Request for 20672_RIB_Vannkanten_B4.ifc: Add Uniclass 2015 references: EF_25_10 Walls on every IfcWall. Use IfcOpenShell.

First a look at what the model holds.

```python
import ifcopenshell

model = ifcopenshell.open("20672_RIB_Vannkanten_B4.ifc")
print(model.schema)
print("classifications:", [c.Name for c in model.by_type("IfcClassification")])
for ifc_class in ("IfcDoor", "IfcRoof", "IfcStair", "IfcWall", "IfcWindow"):
    print(ifc_class, len(model.by_type(ifc_class)))
```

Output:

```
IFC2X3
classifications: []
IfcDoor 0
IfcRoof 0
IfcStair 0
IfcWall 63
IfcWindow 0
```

```python
import ifcopenshell
import ifcopenshell.api.classification

model = ifcopenshell.open("20672_RIB_Vannkanten_B4.ifc")

# IFC2X3 requires Source and Edition and has no link from the project to the system.
system = model.create_entity("IfcClassification", Source="NBS", Edition="2015", Name="Uniclass 2015")

codes = {
    "IfcWall": ("EF_25_10", "Walls"),
}
for ifc_class, (code, name) in codes.items():
    products = model.by_type(ifc_class)
    ifcopenshell.api.classification.add_reference(
        model, products=products, classification=system, identification=code, name=name
    )
    print(code, len(products))

model.write("20672_RIB_Vannkanten_B4_rev.ifc")
```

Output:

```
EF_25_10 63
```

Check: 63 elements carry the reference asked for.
